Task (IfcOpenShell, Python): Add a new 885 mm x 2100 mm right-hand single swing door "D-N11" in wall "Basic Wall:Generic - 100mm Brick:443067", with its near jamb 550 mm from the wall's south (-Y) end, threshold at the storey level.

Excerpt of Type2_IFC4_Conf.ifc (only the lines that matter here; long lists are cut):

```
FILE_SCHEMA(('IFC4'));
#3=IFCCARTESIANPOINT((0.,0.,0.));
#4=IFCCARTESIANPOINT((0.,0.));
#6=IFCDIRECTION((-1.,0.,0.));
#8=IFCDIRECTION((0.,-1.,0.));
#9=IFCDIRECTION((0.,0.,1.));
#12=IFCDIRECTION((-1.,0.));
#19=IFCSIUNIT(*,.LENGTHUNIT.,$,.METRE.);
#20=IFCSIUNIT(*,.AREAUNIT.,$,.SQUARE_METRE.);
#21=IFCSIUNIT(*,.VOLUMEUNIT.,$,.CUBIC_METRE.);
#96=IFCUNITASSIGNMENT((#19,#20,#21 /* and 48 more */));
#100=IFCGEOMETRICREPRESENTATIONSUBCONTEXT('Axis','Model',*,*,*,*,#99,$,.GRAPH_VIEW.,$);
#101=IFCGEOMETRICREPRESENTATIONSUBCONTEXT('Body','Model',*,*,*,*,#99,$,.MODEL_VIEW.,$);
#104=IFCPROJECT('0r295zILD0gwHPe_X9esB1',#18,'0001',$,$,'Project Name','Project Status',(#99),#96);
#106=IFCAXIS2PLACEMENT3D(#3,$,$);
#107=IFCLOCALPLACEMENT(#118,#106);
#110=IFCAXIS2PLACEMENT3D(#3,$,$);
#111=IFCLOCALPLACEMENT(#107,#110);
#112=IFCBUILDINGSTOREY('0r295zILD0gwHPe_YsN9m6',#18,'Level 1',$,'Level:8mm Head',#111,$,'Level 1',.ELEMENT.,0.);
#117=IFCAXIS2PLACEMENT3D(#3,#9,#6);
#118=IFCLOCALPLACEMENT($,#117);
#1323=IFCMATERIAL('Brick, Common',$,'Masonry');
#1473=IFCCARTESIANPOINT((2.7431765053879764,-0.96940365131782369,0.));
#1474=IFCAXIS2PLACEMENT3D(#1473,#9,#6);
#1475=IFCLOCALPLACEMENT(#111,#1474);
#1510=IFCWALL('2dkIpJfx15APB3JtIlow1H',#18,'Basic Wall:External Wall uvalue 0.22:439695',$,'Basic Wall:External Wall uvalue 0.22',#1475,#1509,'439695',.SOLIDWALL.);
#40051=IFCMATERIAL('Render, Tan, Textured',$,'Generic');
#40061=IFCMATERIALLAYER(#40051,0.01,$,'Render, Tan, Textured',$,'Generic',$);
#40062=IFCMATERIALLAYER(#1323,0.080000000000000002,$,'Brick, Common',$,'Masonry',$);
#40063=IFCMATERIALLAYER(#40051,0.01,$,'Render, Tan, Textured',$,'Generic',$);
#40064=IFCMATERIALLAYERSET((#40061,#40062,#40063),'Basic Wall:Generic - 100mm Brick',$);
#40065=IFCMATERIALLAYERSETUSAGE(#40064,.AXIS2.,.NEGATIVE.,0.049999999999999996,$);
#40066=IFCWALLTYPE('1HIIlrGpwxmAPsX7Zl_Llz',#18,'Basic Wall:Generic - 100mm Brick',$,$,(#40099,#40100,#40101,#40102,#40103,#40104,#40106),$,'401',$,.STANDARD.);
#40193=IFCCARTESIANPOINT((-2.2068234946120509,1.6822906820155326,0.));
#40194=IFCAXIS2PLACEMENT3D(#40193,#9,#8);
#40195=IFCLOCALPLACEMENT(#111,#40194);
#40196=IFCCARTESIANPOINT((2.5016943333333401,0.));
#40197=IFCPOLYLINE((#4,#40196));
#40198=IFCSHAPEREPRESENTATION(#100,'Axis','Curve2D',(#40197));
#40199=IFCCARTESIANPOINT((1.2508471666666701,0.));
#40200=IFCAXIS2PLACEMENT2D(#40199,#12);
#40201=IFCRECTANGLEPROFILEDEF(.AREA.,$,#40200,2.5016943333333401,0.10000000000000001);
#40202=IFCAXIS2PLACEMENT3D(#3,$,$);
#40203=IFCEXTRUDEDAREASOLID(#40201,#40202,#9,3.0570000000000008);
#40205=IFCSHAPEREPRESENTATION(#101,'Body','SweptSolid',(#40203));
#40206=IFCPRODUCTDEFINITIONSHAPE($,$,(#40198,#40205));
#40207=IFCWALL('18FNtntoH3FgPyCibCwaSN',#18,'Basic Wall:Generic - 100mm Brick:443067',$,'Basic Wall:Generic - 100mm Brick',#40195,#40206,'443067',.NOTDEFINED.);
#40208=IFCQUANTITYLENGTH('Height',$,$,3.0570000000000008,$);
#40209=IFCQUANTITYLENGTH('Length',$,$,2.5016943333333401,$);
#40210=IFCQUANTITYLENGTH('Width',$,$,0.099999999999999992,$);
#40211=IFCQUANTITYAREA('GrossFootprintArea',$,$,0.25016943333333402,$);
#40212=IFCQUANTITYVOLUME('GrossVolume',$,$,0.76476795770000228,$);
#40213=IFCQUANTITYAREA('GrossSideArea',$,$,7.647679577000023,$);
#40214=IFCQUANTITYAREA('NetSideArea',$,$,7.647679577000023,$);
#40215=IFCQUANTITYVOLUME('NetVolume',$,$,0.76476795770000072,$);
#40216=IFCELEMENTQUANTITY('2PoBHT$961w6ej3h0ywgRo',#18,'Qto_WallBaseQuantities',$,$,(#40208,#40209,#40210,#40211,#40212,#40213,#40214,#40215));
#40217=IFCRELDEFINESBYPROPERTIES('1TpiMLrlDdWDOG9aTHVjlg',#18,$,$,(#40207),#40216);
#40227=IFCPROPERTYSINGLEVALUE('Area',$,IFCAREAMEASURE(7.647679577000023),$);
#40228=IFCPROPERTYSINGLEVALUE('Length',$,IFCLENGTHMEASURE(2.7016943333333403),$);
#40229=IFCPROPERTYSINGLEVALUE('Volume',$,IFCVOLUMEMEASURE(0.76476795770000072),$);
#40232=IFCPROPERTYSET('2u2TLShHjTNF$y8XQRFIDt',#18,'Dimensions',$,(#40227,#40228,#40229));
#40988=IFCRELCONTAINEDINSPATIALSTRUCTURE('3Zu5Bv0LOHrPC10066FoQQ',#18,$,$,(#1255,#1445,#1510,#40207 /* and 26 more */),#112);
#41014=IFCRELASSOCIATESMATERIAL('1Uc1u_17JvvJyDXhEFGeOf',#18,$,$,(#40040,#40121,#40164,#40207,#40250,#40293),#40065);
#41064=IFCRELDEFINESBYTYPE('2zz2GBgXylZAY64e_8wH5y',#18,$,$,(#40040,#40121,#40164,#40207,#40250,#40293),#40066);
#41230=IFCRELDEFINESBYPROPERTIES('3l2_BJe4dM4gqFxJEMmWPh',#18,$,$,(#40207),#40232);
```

```python
import numpy as np
import ifcopenshell
import ifcopenshell.api.feature
import ifcopenshell.api.geometry
import ifcopenshell.api.pset
import ifcopenshell.api.root
import ifcopenshell.api.spatial
import ifcopenshell.geom
import ifcopenshell.util.element
import ifcopenshell.util.placement
import ifcopenshell.util.representation
import ifcopenshell.util.shape
import ifcopenshell.util.unit

model = ifcopenshell.open("Type2_IFC4_Conf.ifc")
unit_scale = ifcopenshell.util.unit.calculate_unit_scale(model)
area_scale = ifcopenshell.util.unit.calculate_unit_scale(model, "AREAUNIT")
volume_scale = ifcopenshell.util.unit.calculate_unit_scale(model, "VOLUMEUNIT")
settings = ifcopenshell.geom.settings()


def volume(element):
    """Net volume in cubic metres, openings subtracted."""
    shape = ifcopenshell.geom.create_shape(settings, element)
    return ifcopenshell.util.shape.get_volume(shape.geometry)


wall = model.by_guid("18FNtntoH3FgPyCibCwaSN")
storey = ifcopenshell.util.element.get_container(wall, ifc_class="IfcBuildingStorey")
context = ifcopenshell.util.representation.get_context(model, "Model", "Body", "MODEL_VIEW")
before = volume(wall)

width, height, from_end, sill = 0.885, 2.1, 0.55, 0.0  # metres

# The wall runs along its own X axis, and the end named is its -X end.
wall_shape = ifcopenshell.geom.create_shape(settings, wall)
x, y, z = ifcopenshell.util.shape.get_vertices(wall_shape.geometry).T
start = x.min() + from_end
face, thickness = float(y.min()), float(y.max() - y.min())
wall_matrix = ifcopenshell.util.placement.get_local_placement(wall.ObjectPlacement)
level = ifcopenshell.util.placement.get_local_placement(storey.ObjectPlacement)[2, 3]


def in_wall(x, y):
    """Placement at x, y metres in the wall's axes, at sill height."""
    matrix = wall_matrix.copy()
    matrix[:, 3] = wall_matrix @ np.array([x / unit_scale, y / unit_scale, 0.0, 1.0])
    matrix[2, 3] = level + sill / unit_scale
    return matrix


# Opening: a box that overshoots both wall faces by 50 mm.
opening = ifcopenshell.api.root.create_entity(model, ifc_class="IfcOpeningElement", predefined_type="OPENING")
box = ifcopenshell.api.geometry.add_wall_representation(
    model, context=context, length=width, height=height, thickness=thickness + 0.1
)
ifcopenshell.api.geometry.assign_representation(model, product=opening, representation=box)
ifcopenshell.api.geometry.edit_object_placement(model, product=opening, matrix=in_wall(start, face - 0.05), is_si=False)
ifcopenshell.api.feature.add_feature(model, feature=opening, element=wall)

door = ifcopenshell.api.root.create_entity(model, ifc_class="IfcDoor", name="D-N11", predefined_type="DOOR")
door.OverallWidth, door.OverallHeight = width / unit_scale, height / unit_scale
door.OperationType = "SINGLE_SWING_RIGHT"
body = ifcopenshell.api.geometry.add_door_representation(
    model,
    context=context,
    overall_width=door.OverallWidth,
    overall_height=door.OverallHeight,
    operation_type="SINGLE_SWING_RIGHT",
    lining_properties={"LiningDepth": thickness / unit_scale, "ThresholdDepth": thickness / unit_scale},
)
ifcopenshell.api.geometry.assign_representation(model, product=door, representation=body)
ifcopenshell.api.spatial.assign_container(model, products=[door], relating_structure=storey)
ifcopenshell.api.feature.add_filling(model, opening=opening, element=door)

# The lining spans the wall, so the door starts at the wall face.
ifcopenshell.api.geometry.edit_object_placement(model, product=door, matrix=in_wall(start, face), is_si=False)

after = volume(wall)

# Update the wall's stored quantities.
qto = model.by_id(ifcopenshell.util.element.get_pset(wall, "Qto_WallBaseQuantities", should_inherit=False)["id"])
ifcopenshell.api.pset.edit_qto(model, qto=qto, properties={
    "NetSideArea": after / thickness / area_scale,
    "NetVolume": after / volume_scale,
})
pset = model.by_id(ifcopenshell.util.element.get_pset(wall, "Dimensions", should_inherit=False)["id"])
ifcopenshell.api.pset.edit_pset(model, pset=pset, properties={
    "Area": model.create_entity("IfcAreaMeasure", after / thickness / area_scale),
    "Volume": model.create_entity("IfcVolumeMeasure", after / volume_scale),
})

print(f"wall volume {before:.3f} -> {after:.3f} m3")

model.write("Type2_IFC4_Conf_rev.ifc")
```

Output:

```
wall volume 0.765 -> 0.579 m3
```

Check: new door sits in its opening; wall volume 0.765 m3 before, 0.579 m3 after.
